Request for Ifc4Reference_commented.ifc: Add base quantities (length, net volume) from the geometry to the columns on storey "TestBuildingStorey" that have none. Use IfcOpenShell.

First a look at what the model holds.

```python
import ifcopenshell
import ifcopenshell.util.element
import ifcopenshell.util.unit

model = ifcopenshell.open("Ifc4Reference_commented.ifc")
print(model.schema)
for unit_type in ("LENGTHUNIT", "AREAUNIT", "VOLUMEUNIT"):
    print(unit_type, ifcopenshell.util.unit.calculate_unit_scale(model, unit_type))
storey = next(s for s in model.by_type("IfcBuildingStorey") if s.Name == "TestBuildingStorey")
columns = [e for e in ifcopenshell.util.element.get_decomposition(storey) if e.is_a("IfcColumn")]
for e in sorted(columns, key=lambda e: e.id()):
    print(e.id(), e.is_a(), e.Name, list(ifcopenshell.util.element.get_psets(e, qtos_only=True)), sep=" | ")
```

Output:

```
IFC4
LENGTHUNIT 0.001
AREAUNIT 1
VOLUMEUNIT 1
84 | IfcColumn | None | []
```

```python
import ifcopenshell
import ifcopenshell.api.pset
import ifcopenshell.geom
import ifcopenshell.util.element
import ifcopenshell.util.shape
import ifcopenshell.util.unit

model = ifcopenshell.open("Ifc4Reference_commented.ifc")
unit_scale = ifcopenshell.util.unit.calculate_unit_scale(model)
volume_scale = ifcopenshell.util.unit.calculate_unit_scale(model, "VOLUMEUNIT")
settings = ifcopenshell.geom.settings()

storey = next(s for s in model.by_type("IfcBuildingStorey") if s.Name == "TestBuildingStorey")
columns = [e for e in ifcopenshell.util.element.get_decomposition(storey) if e.is_a("IfcColumn")]

for e in sorted(columns, key=lambda e: e.id()):
    if ifcopenshell.util.element.get_psets(e, qtos_only=True, should_inherit=False):
        continue
    # Geometry comes back in metres, in the element's own axes.
    shape = ifcopenshell.geom.create_shape(settings, e)
    values = {
        "Length": ifcopenshell.util.shape.get_z(shape.geometry) / unit_scale,
        "NetVolume": ifcopenshell.util.shape.get_volume(shape.geometry) / volume_scale,
    }
    qto = ifcopenshell.api.pset.add_qto(model, product=e, name="Qto_ColumnBaseQuantities")
    ifcopenshell.api.pset.edit_qto(model, qto=qto, properties=values)
    print(e.id(), {k: round(v, 3) for k, v in values.items()})

model.write("Ifc4Reference_commented_updated.ifc")
```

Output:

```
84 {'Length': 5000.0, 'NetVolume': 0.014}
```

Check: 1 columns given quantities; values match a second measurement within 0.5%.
